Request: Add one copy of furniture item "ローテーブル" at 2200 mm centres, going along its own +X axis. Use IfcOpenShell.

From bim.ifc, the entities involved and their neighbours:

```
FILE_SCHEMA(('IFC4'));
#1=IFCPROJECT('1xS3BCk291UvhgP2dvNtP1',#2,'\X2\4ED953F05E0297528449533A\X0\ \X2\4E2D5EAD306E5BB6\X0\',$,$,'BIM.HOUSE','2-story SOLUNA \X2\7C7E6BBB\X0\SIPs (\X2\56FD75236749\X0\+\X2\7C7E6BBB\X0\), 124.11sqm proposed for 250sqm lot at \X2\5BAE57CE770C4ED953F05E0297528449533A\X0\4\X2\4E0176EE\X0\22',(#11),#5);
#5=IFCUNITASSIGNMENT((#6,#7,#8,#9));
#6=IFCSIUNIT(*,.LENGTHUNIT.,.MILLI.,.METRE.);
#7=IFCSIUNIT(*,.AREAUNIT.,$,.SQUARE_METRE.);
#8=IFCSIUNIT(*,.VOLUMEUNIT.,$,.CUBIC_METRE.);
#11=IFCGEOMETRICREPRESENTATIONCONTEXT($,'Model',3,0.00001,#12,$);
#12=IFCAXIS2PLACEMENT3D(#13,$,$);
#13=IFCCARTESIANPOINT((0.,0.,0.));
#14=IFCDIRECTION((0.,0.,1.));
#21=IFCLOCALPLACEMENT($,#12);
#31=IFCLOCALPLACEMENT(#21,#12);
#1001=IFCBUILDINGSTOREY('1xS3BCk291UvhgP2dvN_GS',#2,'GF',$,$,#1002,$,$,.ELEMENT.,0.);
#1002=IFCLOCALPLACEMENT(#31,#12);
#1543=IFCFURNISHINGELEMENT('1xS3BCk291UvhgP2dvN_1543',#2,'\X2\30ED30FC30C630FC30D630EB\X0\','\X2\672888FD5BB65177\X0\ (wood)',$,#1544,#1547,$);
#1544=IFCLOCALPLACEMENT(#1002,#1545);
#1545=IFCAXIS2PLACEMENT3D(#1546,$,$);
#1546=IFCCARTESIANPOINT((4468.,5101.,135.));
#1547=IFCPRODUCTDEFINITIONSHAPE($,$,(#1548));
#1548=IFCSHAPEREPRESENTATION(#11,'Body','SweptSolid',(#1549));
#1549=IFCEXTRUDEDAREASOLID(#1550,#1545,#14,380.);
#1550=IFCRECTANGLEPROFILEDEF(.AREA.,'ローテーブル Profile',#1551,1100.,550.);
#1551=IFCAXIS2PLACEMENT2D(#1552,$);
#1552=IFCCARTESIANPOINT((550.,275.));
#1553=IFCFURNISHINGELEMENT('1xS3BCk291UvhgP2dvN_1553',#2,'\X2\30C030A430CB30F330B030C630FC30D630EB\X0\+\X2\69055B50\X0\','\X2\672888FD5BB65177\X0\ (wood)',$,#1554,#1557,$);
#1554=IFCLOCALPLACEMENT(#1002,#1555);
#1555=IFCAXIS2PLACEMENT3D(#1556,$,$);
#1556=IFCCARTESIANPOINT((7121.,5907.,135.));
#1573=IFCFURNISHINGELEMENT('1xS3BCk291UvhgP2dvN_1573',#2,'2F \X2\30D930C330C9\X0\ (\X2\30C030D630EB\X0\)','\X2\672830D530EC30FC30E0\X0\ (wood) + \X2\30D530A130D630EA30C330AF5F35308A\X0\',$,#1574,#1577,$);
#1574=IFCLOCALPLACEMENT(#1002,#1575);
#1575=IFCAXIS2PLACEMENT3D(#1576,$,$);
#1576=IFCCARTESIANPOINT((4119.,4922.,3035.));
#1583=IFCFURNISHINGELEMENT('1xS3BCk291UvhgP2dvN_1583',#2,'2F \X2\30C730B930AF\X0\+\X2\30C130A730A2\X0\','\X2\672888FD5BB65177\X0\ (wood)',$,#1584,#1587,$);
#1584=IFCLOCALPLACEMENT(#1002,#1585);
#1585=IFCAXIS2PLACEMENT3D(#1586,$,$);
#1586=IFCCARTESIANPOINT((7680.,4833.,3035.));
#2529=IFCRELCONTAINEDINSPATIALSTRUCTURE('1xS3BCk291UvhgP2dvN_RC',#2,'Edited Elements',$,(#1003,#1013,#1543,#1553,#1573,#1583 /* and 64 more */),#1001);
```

```python
import ifcopenshell
import ifcopenshell.api.geometry
import ifcopenshell.api.root
import ifcopenshell.util.element
import ifcopenshell.util.placement
import ifcopenshell.util.unit

model = ifcopenshell.open("bim.ifc")
unit_scale = ifcopenshell.util.unit.calculate_unit_scale(model)


def reuse_history(source, copy):
    """copy_class also copies each property set's owner history, people and application; keep the originals."""
    for rel in copy.IsDefinedBy:
        if rel.is_a("IfcRelDefinesByProperties") and (history := rel.RelatingPropertyDefinition.OwnerHistory):
            rel.RelatingPropertyDefinition.OwnerHistory = source.OwnerHistory
            ifcopenshell.util.element.remove_deep2(model, history)


source = model.by_guid("1xS3BCk291UvhgP2dvN_1543")
base = ifcopenshell.util.placement.get_local_placement(source.ObjectPlacement)
step = base[:3, 0] * 2.2 / unit_scale

for i in range(1, 2):
    copy = ifcopenshell.api.root.copy_class(model, product=source)
    copy.Representation = ifcopenshell.util.element.copy_deep(
        model, source.Representation, exclude=["IfcGeometricRepresentationContext", "IfcRepresentationMap"]
    )
    reuse_history(source, copy)
    matrix = base.copy()
    matrix[:3, 3] += i * step
    print("added at", matrix[:3, 3].round(3) + 0.0)
    ifcopenshell.api.geometry.edit_object_placement(model, product=copy, matrix=matrix, is_si=False)

model.write("bim_updated.ifc")
```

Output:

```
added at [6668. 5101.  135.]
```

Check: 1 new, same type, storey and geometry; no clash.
